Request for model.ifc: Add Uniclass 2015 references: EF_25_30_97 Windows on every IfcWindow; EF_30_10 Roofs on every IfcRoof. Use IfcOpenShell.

First a look at what the model holds.

```python
import ifcopenshell

model = ifcopenshell.open("model.ifc")
print(model.schema)
print("classifications:", [c.Name for c in model.by_type("IfcClassification")])
for ifc_class in ("IfcDoor", "IfcRoof", "IfcStair", "IfcWall", "IfcWindow"):
    print(ifc_class, len(model.by_type(ifc_class)))
```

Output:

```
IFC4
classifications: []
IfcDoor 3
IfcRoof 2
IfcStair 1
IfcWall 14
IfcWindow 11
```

```python
import ifcopenshell
import ifcopenshell.api.classification

model = ifcopenshell.open("model.ifc")

system = ifcopenshell.api.classification.add_classification(model, classification="Uniclass 2015")

codes = {
    "IfcWindow": ("EF_25_30_97", "Windows"),
    "IfcRoof": ("EF_30_10", "Roofs"),
}
for ifc_class, (code, name) in codes.items():
    products = model.by_type(ifc_class)
    ifcopenshell.api.classification.add_reference(
        model, products=products, classification=system, identification=code, name=name
    )
    print(code, len(products))

model.write("model_updated.ifc")
```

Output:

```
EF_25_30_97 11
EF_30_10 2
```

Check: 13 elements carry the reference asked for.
